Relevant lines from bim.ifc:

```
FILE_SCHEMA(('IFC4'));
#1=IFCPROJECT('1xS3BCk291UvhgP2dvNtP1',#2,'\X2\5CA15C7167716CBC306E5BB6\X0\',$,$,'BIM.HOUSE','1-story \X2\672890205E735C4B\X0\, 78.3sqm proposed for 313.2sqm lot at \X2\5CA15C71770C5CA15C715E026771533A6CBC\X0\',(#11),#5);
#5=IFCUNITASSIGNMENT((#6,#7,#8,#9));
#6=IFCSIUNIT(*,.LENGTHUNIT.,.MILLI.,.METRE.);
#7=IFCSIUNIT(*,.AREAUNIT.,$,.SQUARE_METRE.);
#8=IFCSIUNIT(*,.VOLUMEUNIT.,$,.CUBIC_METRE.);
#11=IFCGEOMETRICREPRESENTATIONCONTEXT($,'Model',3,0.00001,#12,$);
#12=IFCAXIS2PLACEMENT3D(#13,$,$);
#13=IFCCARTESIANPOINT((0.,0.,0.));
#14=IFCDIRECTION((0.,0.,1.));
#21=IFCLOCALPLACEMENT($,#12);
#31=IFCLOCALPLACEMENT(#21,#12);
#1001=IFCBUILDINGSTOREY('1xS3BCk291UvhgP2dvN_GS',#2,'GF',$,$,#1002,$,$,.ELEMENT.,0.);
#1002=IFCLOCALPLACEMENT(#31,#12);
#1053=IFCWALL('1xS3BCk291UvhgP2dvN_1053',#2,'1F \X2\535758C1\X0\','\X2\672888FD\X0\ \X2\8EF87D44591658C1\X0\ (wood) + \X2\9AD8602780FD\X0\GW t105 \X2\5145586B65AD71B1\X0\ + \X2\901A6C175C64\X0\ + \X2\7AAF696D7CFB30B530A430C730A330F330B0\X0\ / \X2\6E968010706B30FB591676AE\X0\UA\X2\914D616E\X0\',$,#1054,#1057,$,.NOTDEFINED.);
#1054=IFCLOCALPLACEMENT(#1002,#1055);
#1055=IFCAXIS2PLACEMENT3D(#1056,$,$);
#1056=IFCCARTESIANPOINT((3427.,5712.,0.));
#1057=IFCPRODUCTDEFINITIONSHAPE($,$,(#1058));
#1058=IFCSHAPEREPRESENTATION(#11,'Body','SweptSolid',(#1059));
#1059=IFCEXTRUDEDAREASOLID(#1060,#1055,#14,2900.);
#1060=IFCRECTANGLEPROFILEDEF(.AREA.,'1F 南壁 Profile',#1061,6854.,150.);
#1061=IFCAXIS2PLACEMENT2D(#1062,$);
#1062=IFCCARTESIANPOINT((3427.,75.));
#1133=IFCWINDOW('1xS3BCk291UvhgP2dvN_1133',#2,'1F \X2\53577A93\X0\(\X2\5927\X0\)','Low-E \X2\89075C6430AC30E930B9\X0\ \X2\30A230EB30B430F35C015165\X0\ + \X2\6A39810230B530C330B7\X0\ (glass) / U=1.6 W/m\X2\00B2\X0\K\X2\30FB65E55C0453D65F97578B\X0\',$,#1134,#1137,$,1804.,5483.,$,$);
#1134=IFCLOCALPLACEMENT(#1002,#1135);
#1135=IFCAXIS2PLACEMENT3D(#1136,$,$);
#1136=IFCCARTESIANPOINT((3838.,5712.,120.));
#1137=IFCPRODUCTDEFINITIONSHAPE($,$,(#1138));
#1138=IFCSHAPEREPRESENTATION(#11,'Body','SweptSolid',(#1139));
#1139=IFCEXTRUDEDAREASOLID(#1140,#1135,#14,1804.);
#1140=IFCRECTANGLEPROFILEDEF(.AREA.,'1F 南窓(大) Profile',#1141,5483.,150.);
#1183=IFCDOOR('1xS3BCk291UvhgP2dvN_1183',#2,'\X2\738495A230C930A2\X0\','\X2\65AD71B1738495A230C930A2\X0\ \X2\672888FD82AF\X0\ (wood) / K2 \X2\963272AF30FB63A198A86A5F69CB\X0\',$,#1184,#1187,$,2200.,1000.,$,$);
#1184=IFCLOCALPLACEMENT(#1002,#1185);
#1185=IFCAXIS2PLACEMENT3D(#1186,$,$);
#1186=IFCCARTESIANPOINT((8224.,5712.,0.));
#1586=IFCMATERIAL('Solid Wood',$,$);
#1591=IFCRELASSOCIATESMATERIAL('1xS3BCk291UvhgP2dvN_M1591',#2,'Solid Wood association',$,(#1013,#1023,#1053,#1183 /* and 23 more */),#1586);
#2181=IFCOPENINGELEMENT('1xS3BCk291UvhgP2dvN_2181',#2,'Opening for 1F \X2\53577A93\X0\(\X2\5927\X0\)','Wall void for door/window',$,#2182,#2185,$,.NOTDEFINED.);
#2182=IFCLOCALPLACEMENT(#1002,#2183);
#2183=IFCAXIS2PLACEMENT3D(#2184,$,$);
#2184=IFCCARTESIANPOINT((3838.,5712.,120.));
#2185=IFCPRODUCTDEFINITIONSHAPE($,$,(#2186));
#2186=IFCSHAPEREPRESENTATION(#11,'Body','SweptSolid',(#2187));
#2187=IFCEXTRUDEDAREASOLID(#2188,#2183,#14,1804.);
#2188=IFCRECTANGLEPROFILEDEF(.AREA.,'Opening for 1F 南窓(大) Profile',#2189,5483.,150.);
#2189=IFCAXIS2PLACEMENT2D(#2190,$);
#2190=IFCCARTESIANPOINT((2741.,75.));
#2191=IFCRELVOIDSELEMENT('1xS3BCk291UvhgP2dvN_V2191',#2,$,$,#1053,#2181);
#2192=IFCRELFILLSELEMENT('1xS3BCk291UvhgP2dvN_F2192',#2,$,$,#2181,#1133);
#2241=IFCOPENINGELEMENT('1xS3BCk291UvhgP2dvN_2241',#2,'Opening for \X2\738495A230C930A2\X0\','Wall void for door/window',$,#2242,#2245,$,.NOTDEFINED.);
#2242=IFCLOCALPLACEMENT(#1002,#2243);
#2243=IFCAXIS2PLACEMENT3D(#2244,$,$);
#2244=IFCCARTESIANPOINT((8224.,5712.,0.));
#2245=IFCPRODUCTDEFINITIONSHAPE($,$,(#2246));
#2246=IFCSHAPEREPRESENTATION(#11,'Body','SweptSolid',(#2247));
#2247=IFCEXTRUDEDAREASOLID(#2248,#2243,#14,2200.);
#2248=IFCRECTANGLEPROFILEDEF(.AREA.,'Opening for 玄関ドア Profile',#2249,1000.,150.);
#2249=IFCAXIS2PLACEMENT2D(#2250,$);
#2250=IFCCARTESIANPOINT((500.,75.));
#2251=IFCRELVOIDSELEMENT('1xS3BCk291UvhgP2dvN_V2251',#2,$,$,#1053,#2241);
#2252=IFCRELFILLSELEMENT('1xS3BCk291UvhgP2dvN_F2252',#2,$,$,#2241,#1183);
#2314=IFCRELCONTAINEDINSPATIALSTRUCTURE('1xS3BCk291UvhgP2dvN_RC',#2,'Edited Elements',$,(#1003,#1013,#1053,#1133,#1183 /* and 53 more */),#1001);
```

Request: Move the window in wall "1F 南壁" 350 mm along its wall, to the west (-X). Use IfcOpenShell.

```python
import ifcopenshell
import ifcopenshell.api.geometry
import ifcopenshell.util.placement
import ifcopenshell.util.unit

model = ifcopenshell.open("bim.ifc")
unit_scale = ifcopenshell.util.unit.calculate_unit_scale(model)

window = model.by_guid("1xS3BCk291UvhgP2dvN_1133")
opening = window.FillsVoids[0].RelatingOpeningElement
wall = opening.VoidsElements[0].RelatingBuildingElement

wall_matrix = ifcopenshell.util.placement.get_local_placement(wall.ObjectPlacement)
shift = wall_matrix[:3, 0] * -0.35 / unit_scale
before = ifcopenshell.util.placement.get_local_placement(window.ObjectPlacement)[:3, 3].copy()

# The window is not placed relative to its opening, so move both.
for product in (opening, window):
    matrix = ifcopenshell.util.placement.get_local_placement(product.ObjectPlacement)
    matrix[:3, 3] += shift
    ifcopenshell.api.geometry.edit_object_placement(model, product=product, matrix=matrix, is_si=False)

after = ifcopenshell.util.placement.get_local_placement(window.ObjectPlacement)[:3, 3]
print("window moved by", (after - before).round(3) + 0.0)

model.write("bim_updated.ifc")
```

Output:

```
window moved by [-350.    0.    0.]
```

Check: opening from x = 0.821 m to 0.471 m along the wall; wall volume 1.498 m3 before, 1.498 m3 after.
